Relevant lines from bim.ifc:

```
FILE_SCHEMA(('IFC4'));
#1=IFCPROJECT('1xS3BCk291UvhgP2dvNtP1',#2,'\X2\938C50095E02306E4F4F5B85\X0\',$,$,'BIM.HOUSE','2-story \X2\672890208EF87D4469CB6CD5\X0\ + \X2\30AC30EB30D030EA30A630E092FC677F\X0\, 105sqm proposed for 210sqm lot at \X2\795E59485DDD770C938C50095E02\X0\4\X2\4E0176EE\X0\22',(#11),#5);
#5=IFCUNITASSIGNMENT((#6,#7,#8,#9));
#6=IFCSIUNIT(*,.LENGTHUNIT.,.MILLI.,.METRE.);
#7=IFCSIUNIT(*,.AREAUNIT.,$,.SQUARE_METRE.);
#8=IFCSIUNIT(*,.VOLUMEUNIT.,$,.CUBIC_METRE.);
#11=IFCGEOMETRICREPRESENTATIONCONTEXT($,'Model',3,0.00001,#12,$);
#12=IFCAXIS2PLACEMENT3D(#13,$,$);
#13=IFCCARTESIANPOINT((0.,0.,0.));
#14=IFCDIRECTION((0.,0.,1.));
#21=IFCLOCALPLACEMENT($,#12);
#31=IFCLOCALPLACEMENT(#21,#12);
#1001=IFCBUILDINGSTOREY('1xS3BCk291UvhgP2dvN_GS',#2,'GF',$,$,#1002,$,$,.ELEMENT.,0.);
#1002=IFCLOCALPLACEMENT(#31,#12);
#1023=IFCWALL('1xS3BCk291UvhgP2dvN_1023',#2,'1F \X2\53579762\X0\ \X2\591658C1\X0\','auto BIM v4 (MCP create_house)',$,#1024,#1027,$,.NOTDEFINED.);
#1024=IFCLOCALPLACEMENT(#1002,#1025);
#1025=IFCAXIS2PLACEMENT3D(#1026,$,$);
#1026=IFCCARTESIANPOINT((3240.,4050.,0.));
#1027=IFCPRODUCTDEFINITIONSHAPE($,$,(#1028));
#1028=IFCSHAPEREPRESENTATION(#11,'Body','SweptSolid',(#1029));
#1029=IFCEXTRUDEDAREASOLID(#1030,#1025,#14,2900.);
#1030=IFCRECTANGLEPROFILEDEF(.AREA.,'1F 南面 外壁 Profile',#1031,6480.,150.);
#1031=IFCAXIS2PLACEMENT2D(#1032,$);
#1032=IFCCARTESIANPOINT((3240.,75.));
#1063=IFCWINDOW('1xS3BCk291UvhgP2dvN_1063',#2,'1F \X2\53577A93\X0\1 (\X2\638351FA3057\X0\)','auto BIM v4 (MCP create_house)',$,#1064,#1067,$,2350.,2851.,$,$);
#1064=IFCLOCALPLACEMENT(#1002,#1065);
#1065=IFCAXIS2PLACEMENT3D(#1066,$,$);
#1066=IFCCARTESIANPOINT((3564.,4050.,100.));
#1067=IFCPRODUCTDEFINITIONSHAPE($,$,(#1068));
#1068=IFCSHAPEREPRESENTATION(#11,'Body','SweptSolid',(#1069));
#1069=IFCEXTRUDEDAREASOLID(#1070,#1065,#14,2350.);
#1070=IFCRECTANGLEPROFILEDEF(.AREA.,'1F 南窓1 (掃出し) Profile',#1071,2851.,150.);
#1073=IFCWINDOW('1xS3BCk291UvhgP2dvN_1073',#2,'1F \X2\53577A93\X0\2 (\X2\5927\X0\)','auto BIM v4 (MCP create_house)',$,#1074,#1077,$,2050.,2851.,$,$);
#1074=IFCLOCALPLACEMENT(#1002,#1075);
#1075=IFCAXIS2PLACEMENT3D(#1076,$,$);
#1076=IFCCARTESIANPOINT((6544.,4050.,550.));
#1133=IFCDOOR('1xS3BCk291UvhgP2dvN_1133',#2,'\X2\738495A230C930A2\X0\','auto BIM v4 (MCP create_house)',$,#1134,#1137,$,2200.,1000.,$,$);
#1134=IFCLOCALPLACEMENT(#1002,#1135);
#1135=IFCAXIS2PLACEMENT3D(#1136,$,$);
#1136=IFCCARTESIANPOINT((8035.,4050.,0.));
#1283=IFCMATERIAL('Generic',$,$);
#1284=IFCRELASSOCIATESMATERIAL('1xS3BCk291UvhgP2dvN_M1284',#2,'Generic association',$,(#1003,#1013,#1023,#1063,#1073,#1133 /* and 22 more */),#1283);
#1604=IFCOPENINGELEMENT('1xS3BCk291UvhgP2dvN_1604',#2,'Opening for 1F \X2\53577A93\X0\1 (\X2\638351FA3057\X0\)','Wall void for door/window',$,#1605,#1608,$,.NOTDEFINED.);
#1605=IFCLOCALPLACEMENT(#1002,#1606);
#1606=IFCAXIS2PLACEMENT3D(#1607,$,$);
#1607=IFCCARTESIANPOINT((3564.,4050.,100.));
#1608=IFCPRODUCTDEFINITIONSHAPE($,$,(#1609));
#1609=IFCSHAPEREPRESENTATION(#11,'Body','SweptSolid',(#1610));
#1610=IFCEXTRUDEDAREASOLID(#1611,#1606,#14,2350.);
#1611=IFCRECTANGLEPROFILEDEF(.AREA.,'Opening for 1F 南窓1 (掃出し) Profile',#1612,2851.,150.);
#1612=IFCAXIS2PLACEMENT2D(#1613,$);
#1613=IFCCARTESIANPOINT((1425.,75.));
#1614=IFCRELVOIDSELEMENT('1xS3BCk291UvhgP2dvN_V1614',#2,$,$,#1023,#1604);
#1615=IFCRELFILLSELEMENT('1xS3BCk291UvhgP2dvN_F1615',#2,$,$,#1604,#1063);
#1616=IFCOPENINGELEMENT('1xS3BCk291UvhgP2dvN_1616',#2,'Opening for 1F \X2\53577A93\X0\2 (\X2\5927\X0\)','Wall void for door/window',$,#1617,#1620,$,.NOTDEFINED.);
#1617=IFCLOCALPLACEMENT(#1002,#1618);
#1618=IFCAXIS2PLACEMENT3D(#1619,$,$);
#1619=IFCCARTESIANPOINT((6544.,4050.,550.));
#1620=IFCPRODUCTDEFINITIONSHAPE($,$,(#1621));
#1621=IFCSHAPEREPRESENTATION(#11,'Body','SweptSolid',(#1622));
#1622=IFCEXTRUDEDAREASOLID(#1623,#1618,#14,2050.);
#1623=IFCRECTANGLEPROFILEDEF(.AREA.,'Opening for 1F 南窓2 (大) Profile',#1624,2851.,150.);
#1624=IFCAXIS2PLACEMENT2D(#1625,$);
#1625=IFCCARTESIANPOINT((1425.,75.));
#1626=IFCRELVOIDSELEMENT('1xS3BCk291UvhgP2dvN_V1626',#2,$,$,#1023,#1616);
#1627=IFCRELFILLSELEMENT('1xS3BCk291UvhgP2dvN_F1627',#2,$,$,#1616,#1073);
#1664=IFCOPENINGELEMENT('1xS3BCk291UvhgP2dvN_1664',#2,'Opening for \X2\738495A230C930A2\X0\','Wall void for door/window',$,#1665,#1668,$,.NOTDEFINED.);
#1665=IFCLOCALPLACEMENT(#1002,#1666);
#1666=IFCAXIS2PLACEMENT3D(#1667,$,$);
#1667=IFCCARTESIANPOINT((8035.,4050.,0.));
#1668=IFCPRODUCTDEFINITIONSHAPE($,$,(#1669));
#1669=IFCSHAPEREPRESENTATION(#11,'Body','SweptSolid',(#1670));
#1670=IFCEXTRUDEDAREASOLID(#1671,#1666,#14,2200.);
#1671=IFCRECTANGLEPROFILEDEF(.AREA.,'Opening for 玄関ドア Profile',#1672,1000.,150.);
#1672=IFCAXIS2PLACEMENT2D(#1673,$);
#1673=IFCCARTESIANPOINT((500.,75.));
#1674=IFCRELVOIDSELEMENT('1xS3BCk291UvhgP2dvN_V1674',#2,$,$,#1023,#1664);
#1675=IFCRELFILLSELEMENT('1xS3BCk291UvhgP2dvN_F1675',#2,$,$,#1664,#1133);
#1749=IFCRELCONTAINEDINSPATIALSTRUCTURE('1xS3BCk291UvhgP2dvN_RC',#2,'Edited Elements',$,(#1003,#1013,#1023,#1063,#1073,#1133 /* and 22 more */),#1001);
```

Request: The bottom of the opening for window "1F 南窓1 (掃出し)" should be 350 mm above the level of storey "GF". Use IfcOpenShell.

```python
import numpy as np
import ifcopenshell
import ifcopenshell.api.geometry
import ifcopenshell.geom
import ifcopenshell.util.element
import ifcopenshell.util.placement
import ifcopenshell.util.shape
import ifcopenshell.util.unit

model = ifcopenshell.open("bim.ifc")
unit_scale = ifcopenshell.util.unit.calculate_unit_scale(model)

window = model.by_id(1063)
opening = window.FillsVoids[0].RelatingOpeningElement
storey = ifcopenshell.util.element.get_container(window, ifc_class="IfcBuildingStorey")
level = ifcopenshell.util.placement.get_local_placement(storey.ObjectPlacement)[2, 3]

# The opening's origin need not be at the sill, so measure its lowest point.
shape = ifcopenshell.geom.create_shape(ifcopenshell.geom.settings(), opening)
bottom = ifcopenshell.util.shape.get_shape_bottom_elevation(shape, shape.geometry) / unit_scale
dz = level + 350.0 - bottom

shift = np.array([0.0, 0.0, dz])
# The window is not placed relative to its opening, so move both.
for product in (opening, window):
    matrix = ifcopenshell.util.placement.get_local_placement(product.ObjectPlacement)
    matrix[:3, 3] += shift
    ifcopenshell.api.geometry.edit_object_placement(model, product=product, matrix=matrix, is_si=False)

print(f"moved by {dz * unit_scale:+.3f} m")

model.write("bim_edited.ifc")
```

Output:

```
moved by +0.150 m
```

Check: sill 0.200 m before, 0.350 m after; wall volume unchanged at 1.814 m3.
